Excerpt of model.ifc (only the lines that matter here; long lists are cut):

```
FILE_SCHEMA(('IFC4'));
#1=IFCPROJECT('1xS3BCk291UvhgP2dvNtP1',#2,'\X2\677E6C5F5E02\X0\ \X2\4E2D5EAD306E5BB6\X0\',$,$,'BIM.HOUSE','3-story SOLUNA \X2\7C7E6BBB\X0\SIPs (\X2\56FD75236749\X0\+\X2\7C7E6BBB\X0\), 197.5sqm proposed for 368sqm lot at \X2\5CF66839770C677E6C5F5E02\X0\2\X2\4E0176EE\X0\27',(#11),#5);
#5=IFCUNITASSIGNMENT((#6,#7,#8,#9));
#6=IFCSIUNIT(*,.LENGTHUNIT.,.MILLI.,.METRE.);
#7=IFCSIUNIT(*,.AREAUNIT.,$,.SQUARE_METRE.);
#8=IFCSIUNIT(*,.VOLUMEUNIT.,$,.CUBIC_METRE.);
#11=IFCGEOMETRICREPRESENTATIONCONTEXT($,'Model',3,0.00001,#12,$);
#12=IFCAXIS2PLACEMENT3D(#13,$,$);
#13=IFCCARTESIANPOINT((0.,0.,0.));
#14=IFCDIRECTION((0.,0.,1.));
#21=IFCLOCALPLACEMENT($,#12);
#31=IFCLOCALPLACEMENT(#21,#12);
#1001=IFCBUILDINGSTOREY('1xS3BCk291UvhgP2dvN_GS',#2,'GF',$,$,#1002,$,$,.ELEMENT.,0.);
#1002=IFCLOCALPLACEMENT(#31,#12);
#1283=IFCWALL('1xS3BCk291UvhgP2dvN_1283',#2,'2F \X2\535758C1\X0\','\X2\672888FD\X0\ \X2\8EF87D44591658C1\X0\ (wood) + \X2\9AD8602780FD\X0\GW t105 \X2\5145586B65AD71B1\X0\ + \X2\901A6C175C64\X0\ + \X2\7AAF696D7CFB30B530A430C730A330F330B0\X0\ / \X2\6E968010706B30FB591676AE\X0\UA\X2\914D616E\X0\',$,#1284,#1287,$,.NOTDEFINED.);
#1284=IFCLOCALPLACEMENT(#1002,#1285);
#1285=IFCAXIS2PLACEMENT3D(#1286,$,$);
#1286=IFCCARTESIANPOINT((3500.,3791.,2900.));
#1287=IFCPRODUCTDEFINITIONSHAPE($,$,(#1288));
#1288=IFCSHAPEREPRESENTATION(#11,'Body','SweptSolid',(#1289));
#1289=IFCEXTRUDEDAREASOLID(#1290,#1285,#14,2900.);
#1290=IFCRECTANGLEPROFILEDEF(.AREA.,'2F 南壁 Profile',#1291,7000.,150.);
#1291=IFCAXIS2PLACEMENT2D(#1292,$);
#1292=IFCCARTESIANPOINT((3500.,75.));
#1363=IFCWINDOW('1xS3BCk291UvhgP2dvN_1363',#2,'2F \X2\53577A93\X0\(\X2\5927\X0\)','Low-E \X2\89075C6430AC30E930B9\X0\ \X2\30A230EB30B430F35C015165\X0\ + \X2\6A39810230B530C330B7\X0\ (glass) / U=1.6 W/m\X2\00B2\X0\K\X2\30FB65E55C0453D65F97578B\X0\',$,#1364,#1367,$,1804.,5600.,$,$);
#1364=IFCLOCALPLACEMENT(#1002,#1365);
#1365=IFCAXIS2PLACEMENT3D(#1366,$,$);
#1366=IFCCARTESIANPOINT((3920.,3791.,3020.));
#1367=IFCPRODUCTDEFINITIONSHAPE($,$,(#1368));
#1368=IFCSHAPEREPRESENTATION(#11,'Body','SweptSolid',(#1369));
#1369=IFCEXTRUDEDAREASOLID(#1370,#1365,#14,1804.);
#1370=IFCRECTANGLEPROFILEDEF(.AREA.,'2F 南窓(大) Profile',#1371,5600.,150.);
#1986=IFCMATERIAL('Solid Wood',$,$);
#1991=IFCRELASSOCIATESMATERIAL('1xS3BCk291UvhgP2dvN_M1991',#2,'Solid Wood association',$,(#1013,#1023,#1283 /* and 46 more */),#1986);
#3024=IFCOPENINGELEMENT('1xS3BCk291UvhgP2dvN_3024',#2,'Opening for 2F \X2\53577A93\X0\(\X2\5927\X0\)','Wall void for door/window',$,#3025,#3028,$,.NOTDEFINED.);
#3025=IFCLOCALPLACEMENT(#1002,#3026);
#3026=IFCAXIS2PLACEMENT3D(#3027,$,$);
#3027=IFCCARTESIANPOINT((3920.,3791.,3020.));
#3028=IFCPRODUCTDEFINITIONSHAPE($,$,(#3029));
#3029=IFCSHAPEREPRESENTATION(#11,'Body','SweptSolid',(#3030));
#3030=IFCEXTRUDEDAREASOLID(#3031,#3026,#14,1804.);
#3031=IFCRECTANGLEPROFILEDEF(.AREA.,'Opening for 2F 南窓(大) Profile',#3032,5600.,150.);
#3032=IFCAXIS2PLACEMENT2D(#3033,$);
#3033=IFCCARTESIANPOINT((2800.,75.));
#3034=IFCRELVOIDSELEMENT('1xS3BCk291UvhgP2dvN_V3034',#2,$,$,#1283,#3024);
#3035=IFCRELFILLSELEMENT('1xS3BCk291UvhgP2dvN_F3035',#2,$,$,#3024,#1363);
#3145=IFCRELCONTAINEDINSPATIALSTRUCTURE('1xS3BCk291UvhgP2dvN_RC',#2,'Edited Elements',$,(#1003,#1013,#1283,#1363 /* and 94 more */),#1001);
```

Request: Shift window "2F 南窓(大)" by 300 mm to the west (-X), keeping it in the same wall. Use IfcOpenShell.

```python
import ifcopenshell
import ifcopenshell.api.geometry
import ifcopenshell.util.placement
import ifcopenshell.util.unit

model = ifcopenshell.open("model.ifc")
unit_scale = ifcopenshell.util.unit.calculate_unit_scale(model)

window = model.by_guid("1xS3BCk291UvhgP2dvN_1363")
opening = window.FillsVoids[0].RelatingOpeningElement
wall = opening.VoidsElements[0].RelatingBuildingElement

wall_matrix = ifcopenshell.util.placement.get_local_placement(wall.ObjectPlacement)
shift = wall_matrix[:3, 0] * -0.3 / unit_scale
before = ifcopenshell.util.placement.get_local_placement(window.ObjectPlacement)[:3, 3].copy()

# The window is not placed relative to its opening, so move both.
for product in (opening, window):
    matrix = ifcopenshell.util.placement.get_local_placement(product.ObjectPlacement)
    matrix[:3, 3] += shift
    ifcopenshell.api.geometry.edit_object_placement(model, product=product, matrix=matrix, is_si=False)

after = ifcopenshell.util.placement.get_local_placement(window.ObjectPlacement)[:3, 3]
print("window moved by", (after - before).round(3) + 0.0)

model.write("model_updated.ifc")
```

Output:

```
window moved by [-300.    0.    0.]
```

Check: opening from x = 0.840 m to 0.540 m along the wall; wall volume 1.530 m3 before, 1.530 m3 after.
